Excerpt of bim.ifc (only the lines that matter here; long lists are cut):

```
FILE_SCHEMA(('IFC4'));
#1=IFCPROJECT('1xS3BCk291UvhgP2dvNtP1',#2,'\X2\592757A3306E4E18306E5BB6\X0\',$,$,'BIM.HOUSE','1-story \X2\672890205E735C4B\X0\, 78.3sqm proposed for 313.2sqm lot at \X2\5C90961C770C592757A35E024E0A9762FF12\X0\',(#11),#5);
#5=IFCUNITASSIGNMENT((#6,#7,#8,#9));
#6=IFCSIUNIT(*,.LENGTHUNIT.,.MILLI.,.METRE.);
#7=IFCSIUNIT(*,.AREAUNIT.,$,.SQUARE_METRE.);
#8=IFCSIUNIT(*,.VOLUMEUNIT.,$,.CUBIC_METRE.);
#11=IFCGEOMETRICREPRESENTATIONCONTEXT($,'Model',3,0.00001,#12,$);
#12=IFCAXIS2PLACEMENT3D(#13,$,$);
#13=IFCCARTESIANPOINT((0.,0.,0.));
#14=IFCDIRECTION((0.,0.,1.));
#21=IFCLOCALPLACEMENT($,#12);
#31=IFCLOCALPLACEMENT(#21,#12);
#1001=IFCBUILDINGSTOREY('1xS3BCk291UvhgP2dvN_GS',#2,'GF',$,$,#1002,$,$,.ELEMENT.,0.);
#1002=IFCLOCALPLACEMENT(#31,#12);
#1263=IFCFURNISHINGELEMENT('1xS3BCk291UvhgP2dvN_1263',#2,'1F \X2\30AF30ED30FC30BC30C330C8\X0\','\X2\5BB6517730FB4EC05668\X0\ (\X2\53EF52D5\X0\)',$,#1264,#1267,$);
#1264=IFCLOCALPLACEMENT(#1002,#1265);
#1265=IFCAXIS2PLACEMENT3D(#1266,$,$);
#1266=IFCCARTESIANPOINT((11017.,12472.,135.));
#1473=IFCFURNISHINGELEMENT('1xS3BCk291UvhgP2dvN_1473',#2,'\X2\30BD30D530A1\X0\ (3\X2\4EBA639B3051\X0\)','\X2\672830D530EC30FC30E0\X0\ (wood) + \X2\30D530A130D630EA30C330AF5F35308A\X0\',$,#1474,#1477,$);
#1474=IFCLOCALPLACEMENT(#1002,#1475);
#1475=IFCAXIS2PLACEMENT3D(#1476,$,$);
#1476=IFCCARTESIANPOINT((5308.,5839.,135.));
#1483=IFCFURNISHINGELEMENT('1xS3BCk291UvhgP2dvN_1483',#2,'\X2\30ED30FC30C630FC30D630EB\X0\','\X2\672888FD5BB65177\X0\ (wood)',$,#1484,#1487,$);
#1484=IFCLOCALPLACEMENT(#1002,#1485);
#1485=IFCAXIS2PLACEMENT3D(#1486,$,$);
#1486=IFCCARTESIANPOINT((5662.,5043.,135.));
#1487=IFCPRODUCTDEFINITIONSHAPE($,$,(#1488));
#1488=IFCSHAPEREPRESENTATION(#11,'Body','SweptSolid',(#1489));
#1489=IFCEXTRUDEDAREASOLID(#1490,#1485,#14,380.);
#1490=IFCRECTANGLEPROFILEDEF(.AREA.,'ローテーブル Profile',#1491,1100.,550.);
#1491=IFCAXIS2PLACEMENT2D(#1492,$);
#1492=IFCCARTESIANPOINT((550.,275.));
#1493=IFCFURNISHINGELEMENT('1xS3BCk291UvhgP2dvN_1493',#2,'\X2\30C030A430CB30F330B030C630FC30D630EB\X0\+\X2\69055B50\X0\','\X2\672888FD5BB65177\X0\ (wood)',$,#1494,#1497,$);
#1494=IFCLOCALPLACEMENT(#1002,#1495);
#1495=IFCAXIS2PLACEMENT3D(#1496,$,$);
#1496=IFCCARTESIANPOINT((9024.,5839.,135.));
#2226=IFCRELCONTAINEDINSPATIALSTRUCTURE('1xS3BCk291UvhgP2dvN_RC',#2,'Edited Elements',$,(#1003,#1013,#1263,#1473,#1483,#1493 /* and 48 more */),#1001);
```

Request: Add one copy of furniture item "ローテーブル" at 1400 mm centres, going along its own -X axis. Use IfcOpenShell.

```python
import ifcopenshell
import ifcopenshell.api.geometry
import ifcopenshell.api.root
import ifcopenshell.util.element
import ifcopenshell.util.placement
import ifcopenshell.util.unit

model = ifcopenshell.open("bim.ifc")
unit_scale = ifcopenshell.util.unit.calculate_unit_scale(model)


def reuse_history(source, copy):
    """copy_class also copies each property set's owner history, people and application; keep the originals."""
    for rel in copy.IsDefinedBy:
        if rel.is_a("IfcRelDefinesByProperties") and (history := rel.RelatingPropertyDefinition.OwnerHistory):
            rel.RelatingPropertyDefinition.OwnerHistory = source.OwnerHistory
            ifcopenshell.util.element.remove_deep2(model, history)


source = model.by_id(1483)
base = ifcopenshell.util.placement.get_local_placement(source.ObjectPlacement)
step = -base[:3, 0] * 1.4 / unit_scale

for i in range(1, 2):
    copy = ifcopenshell.api.root.copy_class(model, product=source)
    copy.Representation = ifcopenshell.util.element.copy_deep(
        model, source.Representation, exclude=["IfcGeometricRepresentationContext", "IfcRepresentationMap"]
    )
    reuse_history(source, copy)
    matrix = base.copy()
    matrix[:3, 3] += i * step
    print("added at", matrix[:3, 3].round(3) + 0.0)
    ifcopenshell.api.geometry.edit_object_placement(model, product=copy, matrix=matrix, is_si=False)

model.write("bim_edited.ifc")
```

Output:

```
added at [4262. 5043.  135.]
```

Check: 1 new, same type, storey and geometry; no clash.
